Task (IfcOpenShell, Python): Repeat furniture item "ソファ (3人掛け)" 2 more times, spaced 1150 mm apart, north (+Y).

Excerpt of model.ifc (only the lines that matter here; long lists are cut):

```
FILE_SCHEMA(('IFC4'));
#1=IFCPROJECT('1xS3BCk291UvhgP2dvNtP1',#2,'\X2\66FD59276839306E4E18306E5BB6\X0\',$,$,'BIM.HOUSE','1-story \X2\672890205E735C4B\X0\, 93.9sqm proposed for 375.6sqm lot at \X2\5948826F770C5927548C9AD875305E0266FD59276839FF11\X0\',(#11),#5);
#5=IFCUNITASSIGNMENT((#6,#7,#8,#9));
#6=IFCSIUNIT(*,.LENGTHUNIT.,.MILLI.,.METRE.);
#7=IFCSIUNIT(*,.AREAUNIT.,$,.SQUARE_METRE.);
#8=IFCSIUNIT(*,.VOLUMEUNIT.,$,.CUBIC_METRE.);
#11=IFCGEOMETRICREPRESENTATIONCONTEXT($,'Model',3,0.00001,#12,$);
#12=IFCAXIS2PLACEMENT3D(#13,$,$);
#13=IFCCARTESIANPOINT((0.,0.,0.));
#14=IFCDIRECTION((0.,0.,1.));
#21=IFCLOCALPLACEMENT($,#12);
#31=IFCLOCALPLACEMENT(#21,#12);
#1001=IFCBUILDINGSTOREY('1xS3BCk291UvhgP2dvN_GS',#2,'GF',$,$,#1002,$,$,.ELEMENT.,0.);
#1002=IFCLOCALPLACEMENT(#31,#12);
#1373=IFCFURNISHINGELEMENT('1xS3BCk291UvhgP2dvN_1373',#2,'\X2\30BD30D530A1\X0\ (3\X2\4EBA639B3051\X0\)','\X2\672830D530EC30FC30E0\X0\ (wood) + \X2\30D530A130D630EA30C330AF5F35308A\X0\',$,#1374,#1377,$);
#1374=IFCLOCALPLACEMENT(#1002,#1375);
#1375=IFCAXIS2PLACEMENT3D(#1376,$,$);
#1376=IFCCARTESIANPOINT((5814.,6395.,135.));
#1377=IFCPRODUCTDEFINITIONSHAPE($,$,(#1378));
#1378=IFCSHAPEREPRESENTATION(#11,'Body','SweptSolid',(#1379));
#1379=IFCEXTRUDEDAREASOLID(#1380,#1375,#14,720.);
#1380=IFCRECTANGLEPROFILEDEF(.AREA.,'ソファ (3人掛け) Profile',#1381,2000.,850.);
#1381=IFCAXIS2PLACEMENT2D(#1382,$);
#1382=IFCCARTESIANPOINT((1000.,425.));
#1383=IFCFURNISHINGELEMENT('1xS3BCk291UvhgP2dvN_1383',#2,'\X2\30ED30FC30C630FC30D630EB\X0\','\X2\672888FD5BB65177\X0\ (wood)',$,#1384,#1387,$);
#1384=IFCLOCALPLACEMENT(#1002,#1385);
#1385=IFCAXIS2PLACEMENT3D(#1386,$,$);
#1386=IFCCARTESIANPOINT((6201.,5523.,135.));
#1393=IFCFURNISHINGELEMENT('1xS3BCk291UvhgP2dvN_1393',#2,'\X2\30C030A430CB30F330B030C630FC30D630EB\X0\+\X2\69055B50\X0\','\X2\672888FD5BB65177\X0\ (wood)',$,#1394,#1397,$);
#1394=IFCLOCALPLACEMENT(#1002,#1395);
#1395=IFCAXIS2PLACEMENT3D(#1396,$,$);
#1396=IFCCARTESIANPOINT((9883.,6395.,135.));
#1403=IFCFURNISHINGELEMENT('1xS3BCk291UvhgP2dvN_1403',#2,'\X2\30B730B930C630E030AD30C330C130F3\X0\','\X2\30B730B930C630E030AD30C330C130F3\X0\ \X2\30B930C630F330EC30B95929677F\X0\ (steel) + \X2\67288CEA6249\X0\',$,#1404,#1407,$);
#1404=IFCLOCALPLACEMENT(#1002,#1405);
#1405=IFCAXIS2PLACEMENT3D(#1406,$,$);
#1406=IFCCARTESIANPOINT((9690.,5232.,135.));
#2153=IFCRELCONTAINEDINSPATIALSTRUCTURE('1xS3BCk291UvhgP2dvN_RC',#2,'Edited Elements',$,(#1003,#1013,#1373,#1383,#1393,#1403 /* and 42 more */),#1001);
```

```python
import numpy as np
import ifcopenshell
import ifcopenshell.api.geometry
import ifcopenshell.api.root
import ifcopenshell.util.element
import ifcopenshell.util.placement
import ifcopenshell.util.unit

model = ifcopenshell.open("model.ifc")
unit_scale = ifcopenshell.util.unit.calculate_unit_scale(model)


def reuse_history(source, copy):
    """copy_class also copies each property set's owner history, people and application; keep the originals."""
    for rel in copy.IsDefinedBy:
        if rel.is_a("IfcRelDefinesByProperties") and (history := rel.RelatingPropertyDefinition.OwnerHistory):
            rel.RelatingPropertyDefinition.OwnerHistory = source.OwnerHistory
            ifcopenshell.util.element.remove_deep2(model, history)


source = model.by_guid("1xS3BCk291UvhgP2dvN_1373")
base = ifcopenshell.util.placement.get_local_placement(source.ObjectPlacement)
step = np.array([0.0, 1.0, 0.0]) * 1.15 / unit_scale

for i in range(1, 3):
    copy = ifcopenshell.api.root.copy_class(model, product=source)
    copy.Representation = ifcopenshell.util.element.copy_deep(
        model, source.Representation, exclude=["IfcGeometricRepresentationContext", "IfcRepresentationMap"]
    )
    reuse_history(source, copy)
    matrix = base.copy()
    matrix[:3, 3] += i * step
    print("added at", matrix[:3, 3].round(3) + 0.0)
    ifcopenshell.api.geometry.edit_object_placement(model, product=copy, matrix=matrix, is_si=False)

model.write("model_updated.ifc")
```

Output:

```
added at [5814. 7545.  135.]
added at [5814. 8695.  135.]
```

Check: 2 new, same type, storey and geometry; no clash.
